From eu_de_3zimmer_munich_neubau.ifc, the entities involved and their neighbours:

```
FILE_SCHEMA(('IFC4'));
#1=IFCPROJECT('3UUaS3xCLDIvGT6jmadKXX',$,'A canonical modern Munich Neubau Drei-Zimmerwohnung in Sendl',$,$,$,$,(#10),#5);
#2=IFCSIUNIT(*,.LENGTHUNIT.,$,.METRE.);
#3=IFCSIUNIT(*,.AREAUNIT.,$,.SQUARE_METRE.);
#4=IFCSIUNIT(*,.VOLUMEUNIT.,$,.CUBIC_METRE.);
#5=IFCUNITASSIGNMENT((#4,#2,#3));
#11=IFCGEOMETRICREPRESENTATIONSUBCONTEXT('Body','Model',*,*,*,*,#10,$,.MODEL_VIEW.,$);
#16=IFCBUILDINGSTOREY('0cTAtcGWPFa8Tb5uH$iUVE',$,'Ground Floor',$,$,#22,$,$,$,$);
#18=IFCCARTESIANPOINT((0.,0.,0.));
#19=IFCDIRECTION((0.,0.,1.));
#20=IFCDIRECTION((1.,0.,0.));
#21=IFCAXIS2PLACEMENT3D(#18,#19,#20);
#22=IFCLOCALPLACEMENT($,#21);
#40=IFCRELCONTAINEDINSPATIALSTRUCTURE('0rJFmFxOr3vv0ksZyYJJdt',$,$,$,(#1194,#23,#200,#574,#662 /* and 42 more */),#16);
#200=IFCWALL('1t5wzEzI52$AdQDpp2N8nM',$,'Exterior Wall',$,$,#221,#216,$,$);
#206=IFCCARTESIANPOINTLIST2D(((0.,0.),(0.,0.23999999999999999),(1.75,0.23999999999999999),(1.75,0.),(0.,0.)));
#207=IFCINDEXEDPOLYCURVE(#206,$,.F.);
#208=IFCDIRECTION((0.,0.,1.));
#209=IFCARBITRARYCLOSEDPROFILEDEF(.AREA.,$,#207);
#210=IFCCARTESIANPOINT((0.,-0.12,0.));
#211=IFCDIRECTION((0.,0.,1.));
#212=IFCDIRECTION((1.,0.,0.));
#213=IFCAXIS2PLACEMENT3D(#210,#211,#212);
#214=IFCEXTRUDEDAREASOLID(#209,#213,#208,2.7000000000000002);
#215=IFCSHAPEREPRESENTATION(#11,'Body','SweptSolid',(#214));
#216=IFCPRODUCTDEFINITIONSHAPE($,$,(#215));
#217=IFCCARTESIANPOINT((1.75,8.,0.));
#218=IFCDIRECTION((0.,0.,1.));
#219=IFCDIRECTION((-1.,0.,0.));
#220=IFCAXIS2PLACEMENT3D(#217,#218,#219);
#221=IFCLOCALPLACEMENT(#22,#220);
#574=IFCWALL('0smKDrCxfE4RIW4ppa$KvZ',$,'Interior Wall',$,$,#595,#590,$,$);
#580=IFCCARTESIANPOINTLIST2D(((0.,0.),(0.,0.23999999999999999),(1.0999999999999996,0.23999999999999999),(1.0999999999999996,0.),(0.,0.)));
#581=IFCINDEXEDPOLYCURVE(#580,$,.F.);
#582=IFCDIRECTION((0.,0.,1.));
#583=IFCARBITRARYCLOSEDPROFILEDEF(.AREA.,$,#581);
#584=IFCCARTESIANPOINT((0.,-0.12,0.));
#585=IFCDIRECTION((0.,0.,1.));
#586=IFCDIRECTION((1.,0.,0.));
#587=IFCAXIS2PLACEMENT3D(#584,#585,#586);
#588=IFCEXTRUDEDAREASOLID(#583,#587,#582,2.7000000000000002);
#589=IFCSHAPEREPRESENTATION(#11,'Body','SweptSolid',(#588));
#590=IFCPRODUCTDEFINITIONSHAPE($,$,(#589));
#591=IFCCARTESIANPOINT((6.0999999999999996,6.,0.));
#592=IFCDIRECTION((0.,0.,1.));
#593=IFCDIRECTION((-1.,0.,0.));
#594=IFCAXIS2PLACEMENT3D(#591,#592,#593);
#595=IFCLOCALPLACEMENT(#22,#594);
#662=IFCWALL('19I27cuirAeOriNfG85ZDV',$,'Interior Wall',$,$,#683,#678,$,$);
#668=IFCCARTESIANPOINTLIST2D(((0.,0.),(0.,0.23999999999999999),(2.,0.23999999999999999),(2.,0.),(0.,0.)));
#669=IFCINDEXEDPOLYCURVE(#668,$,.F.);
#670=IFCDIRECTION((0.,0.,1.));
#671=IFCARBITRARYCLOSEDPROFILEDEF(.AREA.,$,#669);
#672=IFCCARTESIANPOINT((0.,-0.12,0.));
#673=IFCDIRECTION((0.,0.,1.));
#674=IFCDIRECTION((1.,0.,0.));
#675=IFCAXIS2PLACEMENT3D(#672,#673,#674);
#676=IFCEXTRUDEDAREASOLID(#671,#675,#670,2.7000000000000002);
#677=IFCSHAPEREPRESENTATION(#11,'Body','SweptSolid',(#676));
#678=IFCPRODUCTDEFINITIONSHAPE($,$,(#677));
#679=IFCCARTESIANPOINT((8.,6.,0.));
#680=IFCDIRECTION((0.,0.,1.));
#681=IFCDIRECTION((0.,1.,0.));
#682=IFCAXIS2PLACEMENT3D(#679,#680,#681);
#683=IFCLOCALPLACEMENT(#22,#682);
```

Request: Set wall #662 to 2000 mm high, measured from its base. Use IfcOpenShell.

```python
import ifcopenshell
import ifcopenshell.geom
import ifcopenshell.util.representation
import ifcopenshell.util.shape
import ifcopenshell.util.unit

model = ifcopenshell.open("eu_de_3zimmer_munich_neubau.ifc")
unit_scale = ifcopenshell.util.unit.calculate_unit_scale(model)
settings = ifcopenshell.geom.settings()


def volume(element):
    """Net volume in cubic metres, openings subtracted."""
    shape = ifcopenshell.geom.create_shape(settings, element)
    return ifcopenshell.util.shape.get_volume(shape.geometry)


wall = model.by_guid("19I27cuirAeOriNfG85ZDV")
before = volume(wall)

body = ifcopenshell.util.representation.get_representation(wall, "Model", "Body")
solid = body.Items[0]
old_height = solid.Depth
solid.Depth = 2 / unit_scale
after = volume(wall)

print(f"height {old_height:g} -> {solid.Depth:g}, volume {before:.3f} -> {after:.3f} m3")

model.write("eu_de_3zimmer_munich_neubau_edited.ifc")
```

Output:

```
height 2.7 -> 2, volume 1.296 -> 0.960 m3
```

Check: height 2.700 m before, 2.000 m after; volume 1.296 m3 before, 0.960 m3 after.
